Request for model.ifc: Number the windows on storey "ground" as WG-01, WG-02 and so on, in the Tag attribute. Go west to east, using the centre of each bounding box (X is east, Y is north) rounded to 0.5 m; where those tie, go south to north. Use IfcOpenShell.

First a look at what the model holds.

```python
import ifcopenshell
import ifcopenshell.util.element
import ifcopenshell.util.placement

model = ifcopenshell.open("model.ifc")
print(model.schema)
storey = next(s for s in model.by_type("IfcBuildingStorey") if s.Name == "ground")
windows = [e for e in ifcopenshell.util.element.get_decomposition(storey) if e.is_a("IfcWindow")]
for e in sorted(windows, key=lambda e: e.id()):
    origin = ifcopenshell.util.placement.get_local_placement(e.ObjectPlacement)[:3, 3]
    print(e.id(), e.Tag, e.Name, origin.round(2) + 0.0, sep=" | ")
```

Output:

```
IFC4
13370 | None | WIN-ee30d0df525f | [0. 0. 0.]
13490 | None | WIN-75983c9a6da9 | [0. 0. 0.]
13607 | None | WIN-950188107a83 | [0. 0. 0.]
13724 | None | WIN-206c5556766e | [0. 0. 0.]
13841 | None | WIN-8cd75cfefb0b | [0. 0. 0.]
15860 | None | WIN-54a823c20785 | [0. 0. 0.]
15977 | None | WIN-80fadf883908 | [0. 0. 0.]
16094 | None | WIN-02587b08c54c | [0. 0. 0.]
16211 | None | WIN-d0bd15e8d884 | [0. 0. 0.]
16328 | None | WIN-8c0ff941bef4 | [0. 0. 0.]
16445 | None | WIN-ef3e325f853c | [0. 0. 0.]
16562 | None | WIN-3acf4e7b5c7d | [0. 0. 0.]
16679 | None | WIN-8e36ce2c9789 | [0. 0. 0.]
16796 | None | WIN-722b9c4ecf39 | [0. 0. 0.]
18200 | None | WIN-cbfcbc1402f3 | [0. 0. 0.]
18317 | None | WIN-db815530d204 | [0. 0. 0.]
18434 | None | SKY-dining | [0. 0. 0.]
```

```python
import ifcopenshell
import ifcopenshell.geom
import ifcopenshell.util.element
import ifcopenshell.util.shape

model = ifcopenshell.open("model.ifc")
settings = ifcopenshell.geom.settings()
settings.set("use-world-coords", True)


def centre(element):
    shape = ifcopenshell.geom.create_shape(settings, element)
    return ifcopenshell.util.shape.get_bbox_centroid(shape.geometry)


storey = next(s for s in model.by_type("IfcBuildingStorey") if s.Name == "ground")
windows = [e for e in ifcopenshell.util.element.get_decomposition(storey) if e.is_a("IfcWindow")]

# Insertion points can sit at a corner or the storey origin, so sort by the geometry (in metres).
centres = {e: centre(e) for e in windows}
windows.sort(key=lambda e: (round(centres[e][0] / 0.5), centres[e][1]))

for i, e in enumerate(windows, start=1):
    number = f"WG-{i:02d}"
    e.Tag = number
    print(e.id(), number)

model.write("model_rev.ifc")
```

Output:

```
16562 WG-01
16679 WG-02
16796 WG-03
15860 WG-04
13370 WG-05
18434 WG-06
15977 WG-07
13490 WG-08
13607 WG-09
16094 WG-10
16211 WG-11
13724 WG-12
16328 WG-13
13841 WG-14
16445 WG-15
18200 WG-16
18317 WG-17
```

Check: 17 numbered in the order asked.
